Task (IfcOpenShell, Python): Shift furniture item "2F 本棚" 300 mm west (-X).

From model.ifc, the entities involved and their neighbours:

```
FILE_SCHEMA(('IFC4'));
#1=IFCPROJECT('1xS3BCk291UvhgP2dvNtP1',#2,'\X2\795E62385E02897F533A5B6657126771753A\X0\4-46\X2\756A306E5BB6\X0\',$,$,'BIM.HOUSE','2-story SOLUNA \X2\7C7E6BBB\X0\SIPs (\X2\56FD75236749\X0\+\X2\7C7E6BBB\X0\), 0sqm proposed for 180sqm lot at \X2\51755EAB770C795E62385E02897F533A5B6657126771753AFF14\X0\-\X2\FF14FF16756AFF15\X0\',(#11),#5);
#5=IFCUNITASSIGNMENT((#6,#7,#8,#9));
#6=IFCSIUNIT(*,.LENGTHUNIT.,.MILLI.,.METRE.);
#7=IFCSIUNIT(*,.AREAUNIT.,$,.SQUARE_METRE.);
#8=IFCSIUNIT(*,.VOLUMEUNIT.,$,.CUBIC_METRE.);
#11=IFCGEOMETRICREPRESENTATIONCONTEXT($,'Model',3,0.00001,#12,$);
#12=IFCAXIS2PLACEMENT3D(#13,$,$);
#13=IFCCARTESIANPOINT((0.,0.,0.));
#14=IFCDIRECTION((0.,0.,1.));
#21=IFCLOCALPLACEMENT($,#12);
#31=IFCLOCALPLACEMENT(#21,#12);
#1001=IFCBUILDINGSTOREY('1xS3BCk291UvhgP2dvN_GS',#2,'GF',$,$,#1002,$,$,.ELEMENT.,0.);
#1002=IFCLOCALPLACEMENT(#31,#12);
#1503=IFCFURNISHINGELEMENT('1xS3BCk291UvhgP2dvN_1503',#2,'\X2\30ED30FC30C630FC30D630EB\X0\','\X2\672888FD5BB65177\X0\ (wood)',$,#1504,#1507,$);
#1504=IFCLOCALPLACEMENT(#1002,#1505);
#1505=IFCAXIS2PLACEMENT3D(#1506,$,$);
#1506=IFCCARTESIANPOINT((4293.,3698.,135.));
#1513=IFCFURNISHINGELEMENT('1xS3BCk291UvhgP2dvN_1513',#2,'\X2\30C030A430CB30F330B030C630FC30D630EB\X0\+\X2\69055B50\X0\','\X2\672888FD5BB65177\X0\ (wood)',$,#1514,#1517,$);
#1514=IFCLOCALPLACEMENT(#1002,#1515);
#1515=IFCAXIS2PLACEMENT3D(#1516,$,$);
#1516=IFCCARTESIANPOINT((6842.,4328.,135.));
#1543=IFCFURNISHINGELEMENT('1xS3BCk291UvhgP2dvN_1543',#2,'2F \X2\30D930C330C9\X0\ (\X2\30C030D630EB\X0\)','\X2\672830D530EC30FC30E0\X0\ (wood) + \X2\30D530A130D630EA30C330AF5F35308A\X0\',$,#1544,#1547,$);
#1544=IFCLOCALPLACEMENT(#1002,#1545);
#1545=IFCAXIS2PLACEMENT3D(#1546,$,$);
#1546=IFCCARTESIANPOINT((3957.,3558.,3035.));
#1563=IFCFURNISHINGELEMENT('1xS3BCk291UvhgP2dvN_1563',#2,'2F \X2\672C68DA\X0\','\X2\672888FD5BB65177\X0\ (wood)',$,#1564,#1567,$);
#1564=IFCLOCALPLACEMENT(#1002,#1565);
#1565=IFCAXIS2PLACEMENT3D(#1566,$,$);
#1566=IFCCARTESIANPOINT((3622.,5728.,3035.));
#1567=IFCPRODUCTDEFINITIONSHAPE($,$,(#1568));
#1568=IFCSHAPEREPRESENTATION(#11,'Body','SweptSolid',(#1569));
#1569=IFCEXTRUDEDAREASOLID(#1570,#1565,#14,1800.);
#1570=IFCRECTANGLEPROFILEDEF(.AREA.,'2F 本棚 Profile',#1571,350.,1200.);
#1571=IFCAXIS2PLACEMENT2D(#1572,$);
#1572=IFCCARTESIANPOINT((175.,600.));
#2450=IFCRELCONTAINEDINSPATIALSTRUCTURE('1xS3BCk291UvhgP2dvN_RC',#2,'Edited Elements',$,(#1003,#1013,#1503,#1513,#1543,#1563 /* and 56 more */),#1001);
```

```python
import ifcopenshell
import ifcopenshell.api.geometry
import ifcopenshell.util.placement
import ifcopenshell.util.unit

model = ifcopenshell.open("model.ifc")
unit_scale = ifcopenshell.util.unit.calculate_unit_scale(model)

item = model.by_guid("1xS3BCk291UvhgP2dvN_1563")
matrix = ifcopenshell.util.placement.get_local_placement(item.ObjectPlacement)
matrix[0, 3] -= 0.3 / unit_scale
ifcopenshell.api.geometry.edit_object_placement(model, product=item, matrix=matrix, is_si=False)

print(ifcopenshell.util.placement.get_local_placement(item.ObjectPlacement).round(3) + 0.0)

model.write("model_v2.ifc")
```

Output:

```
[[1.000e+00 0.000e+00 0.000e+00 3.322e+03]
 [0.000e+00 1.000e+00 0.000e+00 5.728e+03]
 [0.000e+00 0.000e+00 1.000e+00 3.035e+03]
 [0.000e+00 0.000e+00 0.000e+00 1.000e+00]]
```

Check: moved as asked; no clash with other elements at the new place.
